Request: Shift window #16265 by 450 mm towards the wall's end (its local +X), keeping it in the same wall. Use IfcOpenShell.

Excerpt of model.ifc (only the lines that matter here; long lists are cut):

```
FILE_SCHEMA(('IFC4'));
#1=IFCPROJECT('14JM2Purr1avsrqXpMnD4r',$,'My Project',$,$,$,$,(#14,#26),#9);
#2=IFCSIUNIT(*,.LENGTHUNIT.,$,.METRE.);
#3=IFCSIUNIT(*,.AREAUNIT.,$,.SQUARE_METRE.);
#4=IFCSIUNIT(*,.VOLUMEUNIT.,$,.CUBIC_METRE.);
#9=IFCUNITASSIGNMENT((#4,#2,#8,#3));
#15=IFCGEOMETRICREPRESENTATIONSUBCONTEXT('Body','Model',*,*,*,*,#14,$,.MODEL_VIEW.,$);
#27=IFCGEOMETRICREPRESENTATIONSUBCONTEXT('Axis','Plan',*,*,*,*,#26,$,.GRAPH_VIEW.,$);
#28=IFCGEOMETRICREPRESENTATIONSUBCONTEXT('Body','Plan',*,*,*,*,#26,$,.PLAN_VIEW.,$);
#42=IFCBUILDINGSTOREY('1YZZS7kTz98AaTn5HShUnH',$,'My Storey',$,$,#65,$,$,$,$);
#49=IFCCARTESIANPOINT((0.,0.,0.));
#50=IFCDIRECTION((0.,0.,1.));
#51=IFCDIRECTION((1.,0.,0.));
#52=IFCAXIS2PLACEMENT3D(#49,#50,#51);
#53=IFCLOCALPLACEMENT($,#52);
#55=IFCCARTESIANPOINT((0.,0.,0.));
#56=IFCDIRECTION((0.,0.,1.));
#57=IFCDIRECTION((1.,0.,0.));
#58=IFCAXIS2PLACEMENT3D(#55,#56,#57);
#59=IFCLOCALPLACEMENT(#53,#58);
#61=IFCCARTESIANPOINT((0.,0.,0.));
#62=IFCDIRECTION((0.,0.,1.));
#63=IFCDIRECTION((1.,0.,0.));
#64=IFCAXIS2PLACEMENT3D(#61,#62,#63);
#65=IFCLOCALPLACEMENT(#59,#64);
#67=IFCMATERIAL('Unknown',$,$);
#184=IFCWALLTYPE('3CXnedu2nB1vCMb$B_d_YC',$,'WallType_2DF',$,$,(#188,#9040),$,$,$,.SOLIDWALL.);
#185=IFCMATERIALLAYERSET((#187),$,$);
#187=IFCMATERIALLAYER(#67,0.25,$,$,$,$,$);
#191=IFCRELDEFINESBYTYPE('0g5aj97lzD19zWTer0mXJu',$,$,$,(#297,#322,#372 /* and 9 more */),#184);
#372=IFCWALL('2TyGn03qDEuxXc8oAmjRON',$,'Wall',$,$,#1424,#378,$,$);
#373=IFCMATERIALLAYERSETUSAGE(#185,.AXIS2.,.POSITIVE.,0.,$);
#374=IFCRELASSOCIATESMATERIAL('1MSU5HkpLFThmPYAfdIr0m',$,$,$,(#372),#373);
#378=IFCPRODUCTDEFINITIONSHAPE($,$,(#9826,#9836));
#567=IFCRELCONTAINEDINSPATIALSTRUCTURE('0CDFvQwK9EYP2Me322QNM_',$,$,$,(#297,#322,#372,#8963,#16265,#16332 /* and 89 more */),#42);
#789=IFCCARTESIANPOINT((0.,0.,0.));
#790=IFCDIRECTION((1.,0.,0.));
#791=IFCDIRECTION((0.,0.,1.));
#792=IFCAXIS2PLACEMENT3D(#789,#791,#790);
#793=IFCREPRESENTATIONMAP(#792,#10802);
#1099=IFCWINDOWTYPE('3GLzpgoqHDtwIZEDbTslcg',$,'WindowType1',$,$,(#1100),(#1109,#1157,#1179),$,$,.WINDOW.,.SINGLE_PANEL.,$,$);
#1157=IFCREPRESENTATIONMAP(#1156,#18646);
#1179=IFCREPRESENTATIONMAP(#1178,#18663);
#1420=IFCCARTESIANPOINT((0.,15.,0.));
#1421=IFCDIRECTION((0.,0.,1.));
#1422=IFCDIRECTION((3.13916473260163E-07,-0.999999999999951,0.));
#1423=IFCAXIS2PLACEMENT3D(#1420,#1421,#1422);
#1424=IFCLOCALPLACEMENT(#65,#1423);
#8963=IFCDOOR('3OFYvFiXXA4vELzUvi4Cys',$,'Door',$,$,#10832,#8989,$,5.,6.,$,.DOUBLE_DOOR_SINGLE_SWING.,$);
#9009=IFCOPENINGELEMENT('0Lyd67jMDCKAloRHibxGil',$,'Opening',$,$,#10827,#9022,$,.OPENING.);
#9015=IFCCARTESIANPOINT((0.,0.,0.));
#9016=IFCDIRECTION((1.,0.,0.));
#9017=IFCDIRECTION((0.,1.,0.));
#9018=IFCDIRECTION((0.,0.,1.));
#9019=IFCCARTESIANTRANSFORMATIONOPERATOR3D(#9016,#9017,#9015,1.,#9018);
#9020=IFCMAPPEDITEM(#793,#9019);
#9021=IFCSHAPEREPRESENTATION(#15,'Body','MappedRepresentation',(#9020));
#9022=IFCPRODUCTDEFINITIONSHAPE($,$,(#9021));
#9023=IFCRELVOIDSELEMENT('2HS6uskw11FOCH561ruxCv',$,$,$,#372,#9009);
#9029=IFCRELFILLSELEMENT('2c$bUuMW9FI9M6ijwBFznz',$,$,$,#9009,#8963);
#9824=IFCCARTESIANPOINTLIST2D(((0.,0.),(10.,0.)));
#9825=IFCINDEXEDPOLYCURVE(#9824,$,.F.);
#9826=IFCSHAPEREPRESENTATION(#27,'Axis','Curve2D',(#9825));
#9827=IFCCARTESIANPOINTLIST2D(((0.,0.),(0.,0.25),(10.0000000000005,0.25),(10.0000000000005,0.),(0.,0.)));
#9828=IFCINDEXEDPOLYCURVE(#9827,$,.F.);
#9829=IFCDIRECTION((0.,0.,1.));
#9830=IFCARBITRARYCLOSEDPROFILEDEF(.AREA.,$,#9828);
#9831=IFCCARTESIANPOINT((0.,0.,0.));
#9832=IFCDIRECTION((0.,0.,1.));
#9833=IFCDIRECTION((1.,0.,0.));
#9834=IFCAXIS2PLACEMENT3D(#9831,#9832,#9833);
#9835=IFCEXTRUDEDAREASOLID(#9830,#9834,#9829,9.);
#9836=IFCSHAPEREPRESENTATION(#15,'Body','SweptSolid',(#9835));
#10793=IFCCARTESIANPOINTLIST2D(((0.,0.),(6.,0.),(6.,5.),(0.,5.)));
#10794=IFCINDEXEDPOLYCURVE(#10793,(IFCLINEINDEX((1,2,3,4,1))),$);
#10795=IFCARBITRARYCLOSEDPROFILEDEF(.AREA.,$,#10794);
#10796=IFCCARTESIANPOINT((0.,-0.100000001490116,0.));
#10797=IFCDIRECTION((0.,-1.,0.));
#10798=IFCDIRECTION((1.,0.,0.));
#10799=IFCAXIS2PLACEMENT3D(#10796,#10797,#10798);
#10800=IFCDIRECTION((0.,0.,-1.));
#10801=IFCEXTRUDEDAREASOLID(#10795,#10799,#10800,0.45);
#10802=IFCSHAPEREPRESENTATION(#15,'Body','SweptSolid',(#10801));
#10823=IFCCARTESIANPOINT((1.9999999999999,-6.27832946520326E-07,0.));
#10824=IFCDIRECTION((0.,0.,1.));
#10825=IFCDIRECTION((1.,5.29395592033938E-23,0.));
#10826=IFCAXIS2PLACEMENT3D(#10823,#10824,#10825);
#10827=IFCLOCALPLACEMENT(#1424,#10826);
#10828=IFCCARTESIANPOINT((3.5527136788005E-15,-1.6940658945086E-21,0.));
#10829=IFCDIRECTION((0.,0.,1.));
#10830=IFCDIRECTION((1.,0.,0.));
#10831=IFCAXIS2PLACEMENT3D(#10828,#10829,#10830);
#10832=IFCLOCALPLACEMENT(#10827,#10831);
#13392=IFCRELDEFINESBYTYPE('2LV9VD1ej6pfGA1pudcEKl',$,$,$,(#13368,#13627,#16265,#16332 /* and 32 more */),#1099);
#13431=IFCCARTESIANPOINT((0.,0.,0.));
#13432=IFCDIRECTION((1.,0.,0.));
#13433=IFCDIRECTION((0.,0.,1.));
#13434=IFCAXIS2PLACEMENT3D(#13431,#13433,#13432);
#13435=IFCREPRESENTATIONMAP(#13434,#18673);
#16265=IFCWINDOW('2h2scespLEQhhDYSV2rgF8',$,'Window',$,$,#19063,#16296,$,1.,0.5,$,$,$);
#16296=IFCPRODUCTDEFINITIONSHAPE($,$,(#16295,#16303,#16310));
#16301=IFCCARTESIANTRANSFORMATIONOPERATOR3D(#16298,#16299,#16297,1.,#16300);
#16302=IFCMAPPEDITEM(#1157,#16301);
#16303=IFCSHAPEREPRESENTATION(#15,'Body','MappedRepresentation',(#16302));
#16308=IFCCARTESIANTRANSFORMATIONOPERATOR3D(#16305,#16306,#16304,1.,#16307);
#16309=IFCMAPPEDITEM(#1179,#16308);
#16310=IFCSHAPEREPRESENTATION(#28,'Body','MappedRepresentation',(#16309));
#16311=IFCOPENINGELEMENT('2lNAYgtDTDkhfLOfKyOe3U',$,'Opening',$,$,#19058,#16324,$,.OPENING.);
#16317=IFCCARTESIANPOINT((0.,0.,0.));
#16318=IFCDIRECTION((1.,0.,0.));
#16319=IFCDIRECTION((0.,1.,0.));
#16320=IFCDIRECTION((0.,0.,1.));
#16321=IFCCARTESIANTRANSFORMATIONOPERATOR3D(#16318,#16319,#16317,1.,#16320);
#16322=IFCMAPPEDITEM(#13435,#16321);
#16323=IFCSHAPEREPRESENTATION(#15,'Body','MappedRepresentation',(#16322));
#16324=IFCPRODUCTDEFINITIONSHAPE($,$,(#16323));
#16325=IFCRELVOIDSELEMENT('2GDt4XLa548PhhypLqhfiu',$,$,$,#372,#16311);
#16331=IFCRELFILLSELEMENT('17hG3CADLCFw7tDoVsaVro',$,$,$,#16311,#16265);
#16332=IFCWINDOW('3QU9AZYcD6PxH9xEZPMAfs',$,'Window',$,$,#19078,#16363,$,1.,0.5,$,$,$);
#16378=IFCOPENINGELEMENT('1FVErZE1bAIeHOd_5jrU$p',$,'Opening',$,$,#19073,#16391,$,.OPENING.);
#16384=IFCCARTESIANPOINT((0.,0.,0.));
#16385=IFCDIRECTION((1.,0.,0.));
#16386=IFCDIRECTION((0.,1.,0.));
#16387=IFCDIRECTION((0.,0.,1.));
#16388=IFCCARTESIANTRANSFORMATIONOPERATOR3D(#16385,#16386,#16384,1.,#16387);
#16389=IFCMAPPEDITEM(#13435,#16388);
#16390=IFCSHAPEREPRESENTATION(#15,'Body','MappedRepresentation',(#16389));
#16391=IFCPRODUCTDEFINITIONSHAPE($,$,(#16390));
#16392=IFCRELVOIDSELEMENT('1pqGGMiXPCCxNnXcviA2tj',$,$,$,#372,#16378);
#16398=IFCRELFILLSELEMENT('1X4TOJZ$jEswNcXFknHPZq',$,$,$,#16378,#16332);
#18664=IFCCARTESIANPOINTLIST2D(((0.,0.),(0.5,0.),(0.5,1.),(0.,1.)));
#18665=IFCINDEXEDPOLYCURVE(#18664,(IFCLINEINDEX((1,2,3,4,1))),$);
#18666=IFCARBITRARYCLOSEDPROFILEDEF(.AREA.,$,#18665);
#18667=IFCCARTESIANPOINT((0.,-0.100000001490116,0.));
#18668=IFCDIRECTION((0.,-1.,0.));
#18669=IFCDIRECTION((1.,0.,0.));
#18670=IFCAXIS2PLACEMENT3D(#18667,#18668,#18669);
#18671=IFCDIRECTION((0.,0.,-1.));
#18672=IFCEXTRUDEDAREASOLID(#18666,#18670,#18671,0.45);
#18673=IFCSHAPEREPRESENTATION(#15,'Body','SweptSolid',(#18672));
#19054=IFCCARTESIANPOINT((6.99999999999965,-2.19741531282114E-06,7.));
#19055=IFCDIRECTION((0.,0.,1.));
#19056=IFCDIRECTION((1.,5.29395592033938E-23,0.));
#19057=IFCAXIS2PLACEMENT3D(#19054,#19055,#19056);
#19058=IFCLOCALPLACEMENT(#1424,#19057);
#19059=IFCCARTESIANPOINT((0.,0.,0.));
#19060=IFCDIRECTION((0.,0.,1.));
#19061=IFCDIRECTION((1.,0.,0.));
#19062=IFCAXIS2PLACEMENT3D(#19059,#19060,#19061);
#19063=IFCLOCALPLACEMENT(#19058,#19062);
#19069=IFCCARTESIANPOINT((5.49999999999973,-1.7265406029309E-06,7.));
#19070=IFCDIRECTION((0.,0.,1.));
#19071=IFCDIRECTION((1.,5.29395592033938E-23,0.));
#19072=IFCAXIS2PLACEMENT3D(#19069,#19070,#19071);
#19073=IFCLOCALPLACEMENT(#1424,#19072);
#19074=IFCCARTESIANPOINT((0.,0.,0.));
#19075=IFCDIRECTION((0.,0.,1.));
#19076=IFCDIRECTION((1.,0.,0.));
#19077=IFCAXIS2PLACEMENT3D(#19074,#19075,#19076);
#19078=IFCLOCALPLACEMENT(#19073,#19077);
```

```python
import ifcopenshell
import ifcopenshell.api.geometry
import ifcopenshell.util.placement

model = ifcopenshell.open("model.ifc")

window = model.by_guid("2h2scespLEQhhDYSV2rgF8")
opening = window.FillsVoids[0].RelatingOpeningElement
wall = opening.VoidsElements[0].RelatingBuildingElement

wall_matrix = ifcopenshell.util.placement.get_local_placement(wall.ObjectPlacement)
shift = wall_matrix[:3, 0] * 0.45
before = ifcopenshell.util.placement.get_local_placement(window.ObjectPlacement)[:3, 3].copy()

# The window is placed relative to its opening, so it follows when the opening moves.
matrix = ifcopenshell.util.placement.get_local_placement(opening.ObjectPlacement)
matrix[:3, 3] += shift
ifcopenshell.api.geometry.edit_object_placement(
    model, product=opening, matrix=matrix, is_si=False, should_transform_children=True
)

after = ifcopenshell.util.placement.get_local_placement(window.ObjectPlacement)[:3, 3]
print("window moved by", (after - before).round(3) + 0.0)

model.write("model_rev.ifc")
```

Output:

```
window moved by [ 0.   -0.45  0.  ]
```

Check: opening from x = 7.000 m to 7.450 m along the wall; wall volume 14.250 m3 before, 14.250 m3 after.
